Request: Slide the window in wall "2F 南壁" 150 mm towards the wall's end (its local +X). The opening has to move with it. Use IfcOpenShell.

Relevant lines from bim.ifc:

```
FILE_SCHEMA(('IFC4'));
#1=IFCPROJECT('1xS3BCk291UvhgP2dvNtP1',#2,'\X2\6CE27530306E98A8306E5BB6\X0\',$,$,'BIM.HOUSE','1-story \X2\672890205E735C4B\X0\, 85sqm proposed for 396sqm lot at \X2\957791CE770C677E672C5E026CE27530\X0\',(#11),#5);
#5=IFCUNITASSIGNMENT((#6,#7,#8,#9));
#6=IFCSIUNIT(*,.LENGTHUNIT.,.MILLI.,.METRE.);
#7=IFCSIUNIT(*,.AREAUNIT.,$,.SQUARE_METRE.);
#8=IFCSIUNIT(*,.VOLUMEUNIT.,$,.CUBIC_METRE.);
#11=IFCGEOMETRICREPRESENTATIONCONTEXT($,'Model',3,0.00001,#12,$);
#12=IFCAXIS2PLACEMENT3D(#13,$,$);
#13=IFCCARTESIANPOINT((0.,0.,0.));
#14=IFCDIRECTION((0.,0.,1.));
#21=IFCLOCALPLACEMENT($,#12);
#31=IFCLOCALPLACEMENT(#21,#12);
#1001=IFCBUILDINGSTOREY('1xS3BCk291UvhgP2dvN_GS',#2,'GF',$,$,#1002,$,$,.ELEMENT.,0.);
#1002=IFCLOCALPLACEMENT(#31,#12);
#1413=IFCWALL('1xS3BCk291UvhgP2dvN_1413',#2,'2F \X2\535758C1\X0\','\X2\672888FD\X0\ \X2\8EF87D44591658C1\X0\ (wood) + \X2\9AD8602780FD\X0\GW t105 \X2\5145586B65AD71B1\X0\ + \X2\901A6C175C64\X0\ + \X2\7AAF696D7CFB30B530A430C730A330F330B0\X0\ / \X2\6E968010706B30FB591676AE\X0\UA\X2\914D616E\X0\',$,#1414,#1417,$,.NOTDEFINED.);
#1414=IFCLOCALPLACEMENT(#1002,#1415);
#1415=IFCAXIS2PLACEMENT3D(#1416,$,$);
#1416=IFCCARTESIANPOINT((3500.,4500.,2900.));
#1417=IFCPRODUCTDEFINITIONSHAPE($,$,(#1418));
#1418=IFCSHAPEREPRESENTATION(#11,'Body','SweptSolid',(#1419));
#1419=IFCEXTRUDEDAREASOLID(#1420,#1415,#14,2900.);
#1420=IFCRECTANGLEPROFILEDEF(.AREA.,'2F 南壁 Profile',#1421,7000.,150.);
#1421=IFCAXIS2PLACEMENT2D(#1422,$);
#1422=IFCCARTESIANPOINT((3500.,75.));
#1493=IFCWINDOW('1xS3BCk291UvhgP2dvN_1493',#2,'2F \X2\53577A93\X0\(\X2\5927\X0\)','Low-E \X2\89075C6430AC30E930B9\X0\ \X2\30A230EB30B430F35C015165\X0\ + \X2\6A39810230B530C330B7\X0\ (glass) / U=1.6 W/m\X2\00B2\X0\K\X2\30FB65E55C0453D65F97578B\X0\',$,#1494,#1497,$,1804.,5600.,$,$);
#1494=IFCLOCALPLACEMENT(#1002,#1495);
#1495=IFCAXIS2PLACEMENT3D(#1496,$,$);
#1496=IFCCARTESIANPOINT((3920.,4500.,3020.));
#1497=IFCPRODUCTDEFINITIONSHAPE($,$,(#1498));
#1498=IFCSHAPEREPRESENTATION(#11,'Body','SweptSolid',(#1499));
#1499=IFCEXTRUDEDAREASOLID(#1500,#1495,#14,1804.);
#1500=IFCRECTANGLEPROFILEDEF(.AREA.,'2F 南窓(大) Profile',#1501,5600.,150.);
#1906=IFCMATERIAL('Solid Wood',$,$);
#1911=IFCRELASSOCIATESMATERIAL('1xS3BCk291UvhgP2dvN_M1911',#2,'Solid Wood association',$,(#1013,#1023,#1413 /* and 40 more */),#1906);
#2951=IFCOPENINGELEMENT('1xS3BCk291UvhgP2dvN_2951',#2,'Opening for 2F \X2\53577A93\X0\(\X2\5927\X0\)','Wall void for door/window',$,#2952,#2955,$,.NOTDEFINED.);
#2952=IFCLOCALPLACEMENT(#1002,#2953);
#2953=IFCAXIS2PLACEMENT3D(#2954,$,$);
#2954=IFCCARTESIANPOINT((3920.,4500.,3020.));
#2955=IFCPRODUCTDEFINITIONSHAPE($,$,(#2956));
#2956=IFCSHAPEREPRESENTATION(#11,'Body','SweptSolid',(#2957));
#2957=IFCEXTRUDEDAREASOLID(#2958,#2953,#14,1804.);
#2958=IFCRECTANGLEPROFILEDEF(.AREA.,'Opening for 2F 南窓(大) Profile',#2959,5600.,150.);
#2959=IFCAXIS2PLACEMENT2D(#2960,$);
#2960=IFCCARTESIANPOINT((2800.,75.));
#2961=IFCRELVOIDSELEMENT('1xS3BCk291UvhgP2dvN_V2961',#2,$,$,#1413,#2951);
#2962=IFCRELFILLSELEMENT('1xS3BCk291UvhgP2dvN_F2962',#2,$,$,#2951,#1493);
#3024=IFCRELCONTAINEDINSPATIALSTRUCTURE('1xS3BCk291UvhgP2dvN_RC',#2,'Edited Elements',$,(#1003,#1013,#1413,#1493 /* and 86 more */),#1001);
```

```python
import ifcopenshell
import ifcopenshell.api.geometry
import ifcopenshell.util.placement
import ifcopenshell.util.unit

model = ifcopenshell.open("bim.ifc")
unit_scale = ifcopenshell.util.unit.calculate_unit_scale(model)

window = model.by_guid("1xS3BCk291UvhgP2dvN_1493")
opening = window.FillsVoids[0].RelatingOpeningElement
wall = opening.VoidsElements[0].RelatingBuildingElement

wall_matrix = ifcopenshell.util.placement.get_local_placement(wall.ObjectPlacement)
shift = wall_matrix[:3, 0] * 0.15 / unit_scale
before = ifcopenshell.util.placement.get_local_placement(window.ObjectPlacement)[:3, 3].copy()

# The window is not placed relative to its opening, so move both.
for product in (opening, window):
    matrix = ifcopenshell.util.placement.get_local_placement(product.ObjectPlacement)
    matrix[:3, 3] += shift
    ifcopenshell.api.geometry.edit_object_placement(model, product=product, matrix=matrix, is_si=False)

after = ifcopenshell.util.placement.get_local_placement(window.ObjectPlacement)[:3, 3]
print("window moved by", (after - before).round(3) + 0.0)

model.write("bim_rev.ifc")
```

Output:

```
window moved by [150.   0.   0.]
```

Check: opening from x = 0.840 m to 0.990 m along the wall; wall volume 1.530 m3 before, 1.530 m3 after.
